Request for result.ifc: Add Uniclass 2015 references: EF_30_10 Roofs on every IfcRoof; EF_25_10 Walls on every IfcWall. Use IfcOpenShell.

First a look at what the model holds.

```python
import ifcopenshell

model = ifcopenshell.open("result.ifc")
print(model.schema)
print("classifications:", [c.Name for c in model.by_type("IfcClassification")])
for ifc_class in ("IfcDoor", "IfcRoof", "IfcStair", "IfcWall", "IfcWindow"):
    print(ifc_class, len(model.by_type(ifc_class)))
```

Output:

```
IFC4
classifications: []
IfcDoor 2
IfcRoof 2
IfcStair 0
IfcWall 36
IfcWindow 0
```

```python
import ifcopenshell
import ifcopenshell.api.classification

model = ifcopenshell.open("result.ifc")

system = ifcopenshell.api.classification.add_classification(model, classification="Uniclass 2015")

codes = {
    "IfcRoof": ("EF_30_10", "Roofs"),
    "IfcWall": ("EF_25_10", "Walls"),
}
for ifc_class, (code, name) in codes.items():
    products = model.by_type(ifc_class)
    ifcopenshell.api.classification.add_reference(
        model, products=products, classification=system, identification=code, name=name
    )
    print(code, len(products))

model.write("result_updated.ifc")
```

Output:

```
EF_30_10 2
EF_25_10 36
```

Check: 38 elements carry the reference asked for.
